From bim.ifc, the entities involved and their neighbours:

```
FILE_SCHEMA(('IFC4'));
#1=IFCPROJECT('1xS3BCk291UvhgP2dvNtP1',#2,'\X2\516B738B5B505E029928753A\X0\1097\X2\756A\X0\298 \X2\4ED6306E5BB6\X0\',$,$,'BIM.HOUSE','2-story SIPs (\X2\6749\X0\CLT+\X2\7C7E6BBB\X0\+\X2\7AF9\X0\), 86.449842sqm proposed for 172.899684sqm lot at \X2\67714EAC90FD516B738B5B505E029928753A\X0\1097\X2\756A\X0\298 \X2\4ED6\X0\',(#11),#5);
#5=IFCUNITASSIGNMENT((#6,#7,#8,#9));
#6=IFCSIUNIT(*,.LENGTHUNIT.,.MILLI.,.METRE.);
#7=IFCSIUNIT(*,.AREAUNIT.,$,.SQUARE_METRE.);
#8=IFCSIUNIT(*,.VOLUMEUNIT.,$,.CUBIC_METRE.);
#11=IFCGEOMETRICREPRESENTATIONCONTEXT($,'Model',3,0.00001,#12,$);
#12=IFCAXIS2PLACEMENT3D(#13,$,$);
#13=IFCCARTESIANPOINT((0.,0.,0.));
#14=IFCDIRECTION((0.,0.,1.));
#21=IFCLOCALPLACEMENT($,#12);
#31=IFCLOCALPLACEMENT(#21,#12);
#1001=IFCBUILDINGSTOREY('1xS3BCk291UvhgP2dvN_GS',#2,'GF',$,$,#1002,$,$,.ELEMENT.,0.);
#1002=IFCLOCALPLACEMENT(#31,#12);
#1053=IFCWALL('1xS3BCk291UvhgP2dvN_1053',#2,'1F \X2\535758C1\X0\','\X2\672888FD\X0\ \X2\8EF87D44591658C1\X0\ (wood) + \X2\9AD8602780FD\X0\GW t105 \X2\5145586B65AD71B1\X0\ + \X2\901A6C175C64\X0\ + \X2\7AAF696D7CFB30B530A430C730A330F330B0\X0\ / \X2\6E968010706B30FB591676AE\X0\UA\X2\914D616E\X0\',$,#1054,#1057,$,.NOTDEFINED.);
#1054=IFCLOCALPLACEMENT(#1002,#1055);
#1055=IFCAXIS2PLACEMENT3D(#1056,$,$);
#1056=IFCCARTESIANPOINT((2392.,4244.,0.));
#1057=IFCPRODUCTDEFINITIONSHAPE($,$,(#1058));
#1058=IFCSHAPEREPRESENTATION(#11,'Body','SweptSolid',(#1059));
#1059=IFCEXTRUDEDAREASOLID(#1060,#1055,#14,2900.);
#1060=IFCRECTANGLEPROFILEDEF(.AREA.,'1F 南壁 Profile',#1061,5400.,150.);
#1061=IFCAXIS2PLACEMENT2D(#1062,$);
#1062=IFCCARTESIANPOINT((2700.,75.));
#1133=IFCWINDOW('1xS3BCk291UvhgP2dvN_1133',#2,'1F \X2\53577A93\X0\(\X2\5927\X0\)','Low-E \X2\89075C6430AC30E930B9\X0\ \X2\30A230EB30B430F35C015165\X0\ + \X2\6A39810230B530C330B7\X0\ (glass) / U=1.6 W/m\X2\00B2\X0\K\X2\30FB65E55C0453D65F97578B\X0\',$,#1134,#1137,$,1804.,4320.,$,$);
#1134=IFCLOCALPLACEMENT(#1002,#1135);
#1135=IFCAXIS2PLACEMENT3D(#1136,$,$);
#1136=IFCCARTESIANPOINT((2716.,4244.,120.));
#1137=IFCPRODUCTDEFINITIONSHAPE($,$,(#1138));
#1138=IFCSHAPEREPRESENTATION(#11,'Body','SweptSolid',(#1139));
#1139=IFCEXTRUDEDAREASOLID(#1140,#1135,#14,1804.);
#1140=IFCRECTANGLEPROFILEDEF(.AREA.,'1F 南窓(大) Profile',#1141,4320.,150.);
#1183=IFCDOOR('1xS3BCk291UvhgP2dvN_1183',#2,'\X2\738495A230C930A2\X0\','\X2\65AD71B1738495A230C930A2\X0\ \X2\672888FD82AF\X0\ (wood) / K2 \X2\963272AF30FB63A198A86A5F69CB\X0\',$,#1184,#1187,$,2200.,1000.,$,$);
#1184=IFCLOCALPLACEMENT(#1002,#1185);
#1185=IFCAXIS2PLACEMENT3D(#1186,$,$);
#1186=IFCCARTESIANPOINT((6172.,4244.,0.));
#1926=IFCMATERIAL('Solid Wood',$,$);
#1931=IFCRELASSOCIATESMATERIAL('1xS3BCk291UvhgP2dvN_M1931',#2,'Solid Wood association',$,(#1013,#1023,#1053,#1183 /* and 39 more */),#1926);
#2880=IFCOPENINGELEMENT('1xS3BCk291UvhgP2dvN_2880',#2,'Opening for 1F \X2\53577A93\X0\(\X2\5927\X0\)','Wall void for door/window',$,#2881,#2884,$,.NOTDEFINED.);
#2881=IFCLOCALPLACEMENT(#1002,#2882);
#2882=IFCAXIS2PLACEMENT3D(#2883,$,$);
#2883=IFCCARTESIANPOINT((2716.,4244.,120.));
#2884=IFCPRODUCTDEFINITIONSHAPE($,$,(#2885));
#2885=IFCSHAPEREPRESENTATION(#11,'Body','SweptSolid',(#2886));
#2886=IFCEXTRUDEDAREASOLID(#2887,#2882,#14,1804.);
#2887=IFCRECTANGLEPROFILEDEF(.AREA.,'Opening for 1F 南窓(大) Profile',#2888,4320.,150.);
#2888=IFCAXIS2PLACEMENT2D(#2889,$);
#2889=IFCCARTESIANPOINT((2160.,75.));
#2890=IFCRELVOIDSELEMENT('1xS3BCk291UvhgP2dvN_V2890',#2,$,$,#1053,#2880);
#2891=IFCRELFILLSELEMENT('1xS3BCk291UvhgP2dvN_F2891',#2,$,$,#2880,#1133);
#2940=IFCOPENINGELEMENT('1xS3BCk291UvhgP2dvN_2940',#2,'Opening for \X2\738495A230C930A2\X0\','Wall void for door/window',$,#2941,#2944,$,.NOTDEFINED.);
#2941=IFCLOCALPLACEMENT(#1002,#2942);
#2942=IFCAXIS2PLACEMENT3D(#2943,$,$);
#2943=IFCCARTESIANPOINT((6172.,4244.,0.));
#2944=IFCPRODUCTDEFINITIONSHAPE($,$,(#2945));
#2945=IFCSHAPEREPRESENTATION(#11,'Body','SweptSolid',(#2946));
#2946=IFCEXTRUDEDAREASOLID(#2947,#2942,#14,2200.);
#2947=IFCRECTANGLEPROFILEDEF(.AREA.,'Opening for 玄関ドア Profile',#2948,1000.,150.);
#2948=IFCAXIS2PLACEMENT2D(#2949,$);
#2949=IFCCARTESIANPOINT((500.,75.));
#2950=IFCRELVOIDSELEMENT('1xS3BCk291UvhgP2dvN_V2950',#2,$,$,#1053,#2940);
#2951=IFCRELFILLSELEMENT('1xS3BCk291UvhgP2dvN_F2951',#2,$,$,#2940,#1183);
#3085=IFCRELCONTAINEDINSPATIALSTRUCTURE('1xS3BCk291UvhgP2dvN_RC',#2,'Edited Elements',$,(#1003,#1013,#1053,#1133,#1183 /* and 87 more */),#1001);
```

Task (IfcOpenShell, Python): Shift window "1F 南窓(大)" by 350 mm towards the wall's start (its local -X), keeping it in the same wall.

```python
import ifcopenshell
import ifcopenshell.api.geometry
import ifcopenshell.util.placement
import ifcopenshell.util.unit

model = ifcopenshell.open("bim.ifc")
unit_scale = ifcopenshell.util.unit.calculate_unit_scale(model)

window = model.by_guid("1xS3BCk291UvhgP2dvN_1133")
opening = window.FillsVoids[0].RelatingOpeningElement
wall = opening.VoidsElements[0].RelatingBuildingElement

wall_matrix = ifcopenshell.util.placement.get_local_placement(wall.ObjectPlacement)
shift = wall_matrix[:3, 0] * -0.35 / unit_scale
before = ifcopenshell.util.placement.get_local_placement(window.ObjectPlacement)[:3, 3].copy()

# The window is not placed relative to its opening, so move both.
for product in (opening, window):
    matrix = ifcopenshell.util.placement.get_local_placement(product.ObjectPlacement)
    matrix[:3, 3] += shift
    ifcopenshell.api.geometry.edit_object_placement(model, product=product, matrix=matrix, is_si=False)

after = ifcopenshell.util.placement.get_local_placement(window.ObjectPlacement)[:3, 3]
print("window moved by", (after - before).round(3) + 0.0)

model.write("bim-out.ifc")
```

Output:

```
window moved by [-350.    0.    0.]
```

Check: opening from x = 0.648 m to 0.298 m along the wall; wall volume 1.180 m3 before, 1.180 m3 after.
